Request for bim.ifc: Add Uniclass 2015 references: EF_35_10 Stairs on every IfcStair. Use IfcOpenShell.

First a look at what the model holds.

```python
import ifcopenshell

model = ifcopenshell.open("bim.ifc")
print(model.schema)
print("classifications:", [c.Name for c in model.by_type("IfcClassification")])
for ifc_class in ("IfcDoor", "IfcRoof", "IfcStair", "IfcWall", "IfcWindow"):
    print(ifc_class, len(model.by_type(ifc_class)))
```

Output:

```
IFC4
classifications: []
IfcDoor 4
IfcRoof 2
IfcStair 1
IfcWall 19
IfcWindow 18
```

```python
import ifcopenshell
import ifcopenshell.api.classification

model = ifcopenshell.open("bim.ifc")

system = ifcopenshell.api.classification.add_classification(model, classification="Uniclass 2015")

codes = {
    "IfcStair": ("EF_35_10", "Stairs"),
}
for ifc_class, (code, name) in codes.items():
    products = model.by_type(ifc_class)
    ifcopenshell.api.classification.add_reference(
        model, products=products, classification=system, identification=code, name=name
    )
    print(code, len(products))

model.write("bim_rev.ifc")
```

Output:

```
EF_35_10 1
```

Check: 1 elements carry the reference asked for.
